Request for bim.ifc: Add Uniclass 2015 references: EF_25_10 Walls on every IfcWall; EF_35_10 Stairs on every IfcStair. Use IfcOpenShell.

First a look at what the model holds.

```python
import ifcopenshell

model = ifcopenshell.open("bim.ifc")
print(model.schema)
print("classifications:", [c.Name for c in model.by_type("IfcClassification")])
for ifc_class in ("IfcDoor", "IfcRoof", "IfcStair", "IfcWall", "IfcWindow"):
    print(ifc_class, len(model.by_type(ifc_class)))
```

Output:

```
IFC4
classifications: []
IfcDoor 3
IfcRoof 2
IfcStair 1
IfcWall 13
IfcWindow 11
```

```python
import ifcopenshell
import ifcopenshell.api.classification

model = ifcopenshell.open("bim.ifc")

system = ifcopenshell.api.classification.add_classification(model, classification="Uniclass 2015")

codes = {
    "IfcWall": ("EF_25_10", "Walls"),
    "IfcStair": ("EF_35_10", "Stairs"),
}
for ifc_class, (code, name) in codes.items():
    products = model.by_type(ifc_class)
    ifcopenshell.api.classification.add_reference(
        model, products=products, classification=system, identification=code, name=name
    )
    print(code, len(products))

model.write("bim_rev.ifc")
```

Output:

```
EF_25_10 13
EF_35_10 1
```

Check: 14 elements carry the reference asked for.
